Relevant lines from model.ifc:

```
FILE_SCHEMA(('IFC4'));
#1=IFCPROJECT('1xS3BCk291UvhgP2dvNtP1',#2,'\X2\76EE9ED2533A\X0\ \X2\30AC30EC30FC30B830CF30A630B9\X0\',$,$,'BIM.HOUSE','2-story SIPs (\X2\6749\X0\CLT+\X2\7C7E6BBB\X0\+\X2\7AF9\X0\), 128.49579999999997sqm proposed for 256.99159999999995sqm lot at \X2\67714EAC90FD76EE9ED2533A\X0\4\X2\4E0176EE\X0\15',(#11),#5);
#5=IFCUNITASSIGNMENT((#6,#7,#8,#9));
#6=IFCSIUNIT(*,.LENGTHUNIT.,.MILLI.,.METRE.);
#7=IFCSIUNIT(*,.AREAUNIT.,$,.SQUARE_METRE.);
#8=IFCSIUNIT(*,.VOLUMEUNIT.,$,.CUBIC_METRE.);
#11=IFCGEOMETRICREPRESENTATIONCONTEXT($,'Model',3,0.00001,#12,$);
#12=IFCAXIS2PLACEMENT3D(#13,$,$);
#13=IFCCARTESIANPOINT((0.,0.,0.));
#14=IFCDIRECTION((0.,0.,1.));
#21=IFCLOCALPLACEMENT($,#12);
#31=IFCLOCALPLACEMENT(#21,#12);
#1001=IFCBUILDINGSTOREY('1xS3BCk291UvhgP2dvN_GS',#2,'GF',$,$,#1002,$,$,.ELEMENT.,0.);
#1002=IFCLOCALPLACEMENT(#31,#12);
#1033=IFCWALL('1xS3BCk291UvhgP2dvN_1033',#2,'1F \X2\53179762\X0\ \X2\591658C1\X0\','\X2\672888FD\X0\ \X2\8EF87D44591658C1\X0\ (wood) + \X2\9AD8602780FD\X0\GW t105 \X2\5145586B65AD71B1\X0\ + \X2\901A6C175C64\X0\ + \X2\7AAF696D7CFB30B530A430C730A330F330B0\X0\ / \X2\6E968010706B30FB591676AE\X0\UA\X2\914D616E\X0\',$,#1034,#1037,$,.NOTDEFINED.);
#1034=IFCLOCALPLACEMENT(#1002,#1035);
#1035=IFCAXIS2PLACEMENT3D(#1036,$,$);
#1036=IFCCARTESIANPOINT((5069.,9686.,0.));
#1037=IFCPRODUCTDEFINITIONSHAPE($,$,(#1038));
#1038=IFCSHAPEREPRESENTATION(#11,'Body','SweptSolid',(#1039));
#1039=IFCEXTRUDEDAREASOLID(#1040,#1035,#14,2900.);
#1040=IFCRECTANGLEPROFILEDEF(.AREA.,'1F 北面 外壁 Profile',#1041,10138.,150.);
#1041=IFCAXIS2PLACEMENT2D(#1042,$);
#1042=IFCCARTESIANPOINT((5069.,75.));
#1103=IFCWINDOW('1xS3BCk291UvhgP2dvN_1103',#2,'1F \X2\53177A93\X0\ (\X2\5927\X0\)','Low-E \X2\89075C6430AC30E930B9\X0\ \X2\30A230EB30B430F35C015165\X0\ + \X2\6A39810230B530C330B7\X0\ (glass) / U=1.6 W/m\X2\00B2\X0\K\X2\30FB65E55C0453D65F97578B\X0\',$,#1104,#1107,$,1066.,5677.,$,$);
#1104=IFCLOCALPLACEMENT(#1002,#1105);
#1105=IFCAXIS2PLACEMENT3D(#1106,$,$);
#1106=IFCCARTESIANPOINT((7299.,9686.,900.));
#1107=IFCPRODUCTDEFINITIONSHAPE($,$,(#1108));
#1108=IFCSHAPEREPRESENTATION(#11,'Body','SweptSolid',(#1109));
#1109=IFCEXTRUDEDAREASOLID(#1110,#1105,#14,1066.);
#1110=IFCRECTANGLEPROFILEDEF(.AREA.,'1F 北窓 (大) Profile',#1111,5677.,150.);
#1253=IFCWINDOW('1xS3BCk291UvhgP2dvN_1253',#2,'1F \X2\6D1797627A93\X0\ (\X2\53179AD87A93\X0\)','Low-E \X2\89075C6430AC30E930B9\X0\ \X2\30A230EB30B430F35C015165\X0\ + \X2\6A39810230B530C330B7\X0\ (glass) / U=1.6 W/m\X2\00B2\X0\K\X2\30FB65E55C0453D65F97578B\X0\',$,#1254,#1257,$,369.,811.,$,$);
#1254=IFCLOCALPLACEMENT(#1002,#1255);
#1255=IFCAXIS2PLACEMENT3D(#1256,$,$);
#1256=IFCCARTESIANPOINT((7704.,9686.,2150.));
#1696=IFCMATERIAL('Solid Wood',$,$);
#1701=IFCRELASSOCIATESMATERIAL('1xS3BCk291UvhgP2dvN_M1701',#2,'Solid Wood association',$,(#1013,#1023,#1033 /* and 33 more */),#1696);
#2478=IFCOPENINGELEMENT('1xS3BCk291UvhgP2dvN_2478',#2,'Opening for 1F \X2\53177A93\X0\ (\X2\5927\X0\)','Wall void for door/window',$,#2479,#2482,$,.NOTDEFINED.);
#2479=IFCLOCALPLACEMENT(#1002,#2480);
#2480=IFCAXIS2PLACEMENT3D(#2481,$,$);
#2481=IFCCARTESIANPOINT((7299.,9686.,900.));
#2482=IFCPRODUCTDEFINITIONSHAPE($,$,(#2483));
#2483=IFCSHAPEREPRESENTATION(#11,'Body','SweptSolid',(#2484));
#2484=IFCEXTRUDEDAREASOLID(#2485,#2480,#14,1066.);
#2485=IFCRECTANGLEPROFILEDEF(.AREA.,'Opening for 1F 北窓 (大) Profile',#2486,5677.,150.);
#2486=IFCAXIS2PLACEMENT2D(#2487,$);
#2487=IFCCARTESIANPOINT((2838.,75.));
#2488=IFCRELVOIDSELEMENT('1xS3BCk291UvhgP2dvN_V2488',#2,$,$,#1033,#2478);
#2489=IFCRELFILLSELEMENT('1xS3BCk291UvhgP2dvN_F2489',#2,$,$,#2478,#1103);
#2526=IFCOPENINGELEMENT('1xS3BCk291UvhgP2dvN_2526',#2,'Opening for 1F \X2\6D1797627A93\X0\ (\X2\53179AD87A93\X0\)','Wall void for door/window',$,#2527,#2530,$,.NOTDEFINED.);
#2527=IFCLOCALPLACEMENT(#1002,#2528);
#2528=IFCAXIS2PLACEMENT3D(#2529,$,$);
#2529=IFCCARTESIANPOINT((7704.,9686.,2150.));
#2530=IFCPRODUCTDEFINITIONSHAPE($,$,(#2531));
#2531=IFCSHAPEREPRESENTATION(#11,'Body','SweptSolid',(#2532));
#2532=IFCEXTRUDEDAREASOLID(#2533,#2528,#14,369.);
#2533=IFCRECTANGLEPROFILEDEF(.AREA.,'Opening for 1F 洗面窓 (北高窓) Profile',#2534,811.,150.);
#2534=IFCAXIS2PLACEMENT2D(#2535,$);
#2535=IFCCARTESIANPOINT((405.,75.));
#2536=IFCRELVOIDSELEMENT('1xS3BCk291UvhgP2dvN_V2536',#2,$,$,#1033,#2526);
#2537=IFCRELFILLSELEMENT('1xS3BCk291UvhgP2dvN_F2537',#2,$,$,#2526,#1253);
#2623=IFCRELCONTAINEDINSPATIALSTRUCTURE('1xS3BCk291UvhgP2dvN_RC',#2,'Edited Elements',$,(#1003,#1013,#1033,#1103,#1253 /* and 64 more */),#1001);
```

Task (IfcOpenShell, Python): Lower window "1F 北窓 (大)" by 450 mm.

```python
import numpy as np
import ifcopenshell
import ifcopenshell.api.geometry
import ifcopenshell.util.placement
import ifcopenshell.util.unit

model = ifcopenshell.open("model.ifc")
unit_scale = ifcopenshell.util.unit.calculate_unit_scale(model)

window = model.by_guid("1xS3BCk291UvhgP2dvN_1103")
opening = window.FillsVoids[0].RelatingOpeningElement
dz = -0.45 / unit_scale

shift = np.array([0.0, 0.0, dz])
# The window is not placed relative to its opening, so move both.
for product in (opening, window):
    matrix = ifcopenshell.util.placement.get_local_placement(product.ObjectPlacement)
    matrix[:3, 3] += shift
    ifcopenshell.api.geometry.edit_object_placement(model, product=product, matrix=matrix, is_si=False)

print(f"moved by {dz * unit_scale:+.3f} m")

model.write("model_v2.ifc")
```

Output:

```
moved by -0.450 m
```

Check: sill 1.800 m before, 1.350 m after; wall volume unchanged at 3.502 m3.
